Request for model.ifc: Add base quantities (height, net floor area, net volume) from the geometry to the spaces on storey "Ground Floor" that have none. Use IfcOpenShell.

First a look at what the model holds.

```python
import ifcopenshell
import ifcopenshell.util.element
import ifcopenshell.util.unit

model = ifcopenshell.open("model.ifc")
print(model.schema)
for unit_type in ("LENGTHUNIT", "AREAUNIT", "VOLUMEUNIT"):
    print(unit_type, ifcopenshell.util.unit.calculate_unit_scale(model, unit_type))
storey = next(s for s in model.by_type("IfcBuildingStorey") if s.Name == "Ground Floor")
spaces = [e for e in ifcopenshell.util.element.get_decomposition(storey) if e.is_a("IfcSpace")]
for e in sorted(spaces, key=lambda e: e.id()):
    print(e.id(), e.is_a(), e.Name, list(ifcopenshell.util.element.get_psets(e, qtos_only=True)), sep=" | ")
```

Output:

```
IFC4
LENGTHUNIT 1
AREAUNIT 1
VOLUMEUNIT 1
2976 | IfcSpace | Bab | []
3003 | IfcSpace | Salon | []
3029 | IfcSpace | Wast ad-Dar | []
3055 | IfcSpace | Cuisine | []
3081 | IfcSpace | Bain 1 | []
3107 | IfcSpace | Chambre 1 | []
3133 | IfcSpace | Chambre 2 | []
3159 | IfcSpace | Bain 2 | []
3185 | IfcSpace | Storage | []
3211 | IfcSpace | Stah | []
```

```python
import ifcopenshell
import ifcopenshell.api.pset
import ifcopenshell.geom
import ifcopenshell.util.element
import ifcopenshell.util.shape
import ifcopenshell.util.unit

model = ifcopenshell.open("model.ifc")
unit_scale = ifcopenshell.util.unit.calculate_unit_scale(model)
area_scale = ifcopenshell.util.unit.calculate_unit_scale(model, "AREAUNIT")
volume_scale = ifcopenshell.util.unit.calculate_unit_scale(model, "VOLUMEUNIT")
settings = ifcopenshell.geom.settings()

storey = next(s for s in model.by_type("IfcBuildingStorey") if s.Name == "Ground Floor")
spaces = [e for e in ifcopenshell.util.element.get_decomposition(storey) if e.is_a("IfcSpace")]

for e in sorted(spaces, key=lambda e: e.id()):
    if ifcopenshell.util.element.get_psets(e, qtos_only=True, should_inherit=False):
        continue
    # Geometry comes back in metres, in the element's own axes.
    shape = ifcopenshell.geom.create_shape(settings, e)
    values = {
        "Height": ifcopenshell.util.shape.get_z(shape.geometry) / unit_scale,
        "NetFloorArea": ifcopenshell.util.shape.get_footprint_area(shape.geometry) / area_scale,
        "NetVolume": ifcopenshell.util.shape.get_volume(shape.geometry) / volume_scale,
    }
    qto = ifcopenshell.api.pset.add_qto(model, product=e, name="Qto_SpaceBaseQuantities")
    ifcopenshell.api.pset.edit_qto(model, qto=qto, properties=values)
    print(e.id(), {k: round(v, 3) for k, v in values.items()})

model.write("model_edited.ifc")
```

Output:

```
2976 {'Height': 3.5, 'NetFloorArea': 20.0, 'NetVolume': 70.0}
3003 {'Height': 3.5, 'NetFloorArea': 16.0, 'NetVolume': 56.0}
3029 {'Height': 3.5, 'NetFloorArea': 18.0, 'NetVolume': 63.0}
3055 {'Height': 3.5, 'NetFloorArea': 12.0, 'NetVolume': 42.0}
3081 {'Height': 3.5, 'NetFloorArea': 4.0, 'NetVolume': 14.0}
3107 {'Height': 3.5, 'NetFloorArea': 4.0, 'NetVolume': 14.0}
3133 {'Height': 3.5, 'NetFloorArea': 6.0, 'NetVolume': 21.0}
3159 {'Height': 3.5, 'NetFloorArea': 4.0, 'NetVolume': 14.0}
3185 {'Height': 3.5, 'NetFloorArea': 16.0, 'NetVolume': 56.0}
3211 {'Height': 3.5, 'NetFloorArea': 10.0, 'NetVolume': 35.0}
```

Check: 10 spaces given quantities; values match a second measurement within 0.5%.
